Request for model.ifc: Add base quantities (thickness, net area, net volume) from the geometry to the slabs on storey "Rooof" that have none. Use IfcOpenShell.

First a look at what the model holds.

```python
import ifcopenshell
import ifcopenshell.util.element
import ifcopenshell.util.unit

model = ifcopenshell.open("model.ifc")
print(model.schema)
for unit_type in ("LENGTHUNIT", "AREAUNIT", "VOLUMEUNIT"):
    print(unit_type, ifcopenshell.util.unit.calculate_unit_scale(model, unit_type))
storey = next(s for s in model.by_type("IfcBuildingStorey") if s.Name == "Rooof")
slabs = [e for e in ifcopenshell.util.element.get_decomposition(storey) if e.is_a("IfcSlab")]
for e in sorted(slabs, key=lambda e: e.id()):
    print(e.id(), e.is_a(), e.Name, list(ifcopenshell.util.element.get_psets(e, qtos_only=True)), sep=" | ")
```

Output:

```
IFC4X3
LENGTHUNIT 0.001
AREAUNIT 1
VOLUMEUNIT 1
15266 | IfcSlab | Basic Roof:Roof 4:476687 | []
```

```python
import ifcopenshell
import ifcopenshell.api.pset
import ifcopenshell.geom
import ifcopenshell.util.element
import ifcopenshell.util.shape
import ifcopenshell.util.unit

model = ifcopenshell.open("model.ifc")
unit_scale = ifcopenshell.util.unit.calculate_unit_scale(model)
area_scale = ifcopenshell.util.unit.calculate_unit_scale(model, "AREAUNIT")
volume_scale = ifcopenshell.util.unit.calculate_unit_scale(model, "VOLUMEUNIT")
settings = ifcopenshell.geom.settings()

storey = next(s for s in model.by_type("IfcBuildingStorey") if s.Name == "Rooof")
slabs = [e for e in ifcopenshell.util.element.get_decomposition(storey) if e.is_a("IfcSlab")]

for e in sorted(slabs, key=lambda e: e.id()):
    if ifcopenshell.util.element.get_psets(e, qtos_only=True, should_inherit=False):
        continue
    # Geometry comes back in metres, in the element's own axes.
    shape = ifcopenshell.geom.create_shape(settings, e)
    values = {
        "Width": ifcopenshell.util.shape.get_z(shape.geometry) / unit_scale,
        "NetArea": ifcopenshell.util.shape.get_footprint_area(shape.geometry) / area_scale,
        "NetVolume": ifcopenshell.util.shape.get_volume(shape.geometry) / volume_scale,
    }
    qto = ifcopenshell.api.pset.add_qto(model, product=e, name="Qto_SlabBaseQuantities")
    ifcopenshell.api.pset.edit_qto(model, qto=qto, properties=values)
    print(e.id(), {k: round(v, 3) for k, v in values.items()})

model.write("model_updated.ifc")
```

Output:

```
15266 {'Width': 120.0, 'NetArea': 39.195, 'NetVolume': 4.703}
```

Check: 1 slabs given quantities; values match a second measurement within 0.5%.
